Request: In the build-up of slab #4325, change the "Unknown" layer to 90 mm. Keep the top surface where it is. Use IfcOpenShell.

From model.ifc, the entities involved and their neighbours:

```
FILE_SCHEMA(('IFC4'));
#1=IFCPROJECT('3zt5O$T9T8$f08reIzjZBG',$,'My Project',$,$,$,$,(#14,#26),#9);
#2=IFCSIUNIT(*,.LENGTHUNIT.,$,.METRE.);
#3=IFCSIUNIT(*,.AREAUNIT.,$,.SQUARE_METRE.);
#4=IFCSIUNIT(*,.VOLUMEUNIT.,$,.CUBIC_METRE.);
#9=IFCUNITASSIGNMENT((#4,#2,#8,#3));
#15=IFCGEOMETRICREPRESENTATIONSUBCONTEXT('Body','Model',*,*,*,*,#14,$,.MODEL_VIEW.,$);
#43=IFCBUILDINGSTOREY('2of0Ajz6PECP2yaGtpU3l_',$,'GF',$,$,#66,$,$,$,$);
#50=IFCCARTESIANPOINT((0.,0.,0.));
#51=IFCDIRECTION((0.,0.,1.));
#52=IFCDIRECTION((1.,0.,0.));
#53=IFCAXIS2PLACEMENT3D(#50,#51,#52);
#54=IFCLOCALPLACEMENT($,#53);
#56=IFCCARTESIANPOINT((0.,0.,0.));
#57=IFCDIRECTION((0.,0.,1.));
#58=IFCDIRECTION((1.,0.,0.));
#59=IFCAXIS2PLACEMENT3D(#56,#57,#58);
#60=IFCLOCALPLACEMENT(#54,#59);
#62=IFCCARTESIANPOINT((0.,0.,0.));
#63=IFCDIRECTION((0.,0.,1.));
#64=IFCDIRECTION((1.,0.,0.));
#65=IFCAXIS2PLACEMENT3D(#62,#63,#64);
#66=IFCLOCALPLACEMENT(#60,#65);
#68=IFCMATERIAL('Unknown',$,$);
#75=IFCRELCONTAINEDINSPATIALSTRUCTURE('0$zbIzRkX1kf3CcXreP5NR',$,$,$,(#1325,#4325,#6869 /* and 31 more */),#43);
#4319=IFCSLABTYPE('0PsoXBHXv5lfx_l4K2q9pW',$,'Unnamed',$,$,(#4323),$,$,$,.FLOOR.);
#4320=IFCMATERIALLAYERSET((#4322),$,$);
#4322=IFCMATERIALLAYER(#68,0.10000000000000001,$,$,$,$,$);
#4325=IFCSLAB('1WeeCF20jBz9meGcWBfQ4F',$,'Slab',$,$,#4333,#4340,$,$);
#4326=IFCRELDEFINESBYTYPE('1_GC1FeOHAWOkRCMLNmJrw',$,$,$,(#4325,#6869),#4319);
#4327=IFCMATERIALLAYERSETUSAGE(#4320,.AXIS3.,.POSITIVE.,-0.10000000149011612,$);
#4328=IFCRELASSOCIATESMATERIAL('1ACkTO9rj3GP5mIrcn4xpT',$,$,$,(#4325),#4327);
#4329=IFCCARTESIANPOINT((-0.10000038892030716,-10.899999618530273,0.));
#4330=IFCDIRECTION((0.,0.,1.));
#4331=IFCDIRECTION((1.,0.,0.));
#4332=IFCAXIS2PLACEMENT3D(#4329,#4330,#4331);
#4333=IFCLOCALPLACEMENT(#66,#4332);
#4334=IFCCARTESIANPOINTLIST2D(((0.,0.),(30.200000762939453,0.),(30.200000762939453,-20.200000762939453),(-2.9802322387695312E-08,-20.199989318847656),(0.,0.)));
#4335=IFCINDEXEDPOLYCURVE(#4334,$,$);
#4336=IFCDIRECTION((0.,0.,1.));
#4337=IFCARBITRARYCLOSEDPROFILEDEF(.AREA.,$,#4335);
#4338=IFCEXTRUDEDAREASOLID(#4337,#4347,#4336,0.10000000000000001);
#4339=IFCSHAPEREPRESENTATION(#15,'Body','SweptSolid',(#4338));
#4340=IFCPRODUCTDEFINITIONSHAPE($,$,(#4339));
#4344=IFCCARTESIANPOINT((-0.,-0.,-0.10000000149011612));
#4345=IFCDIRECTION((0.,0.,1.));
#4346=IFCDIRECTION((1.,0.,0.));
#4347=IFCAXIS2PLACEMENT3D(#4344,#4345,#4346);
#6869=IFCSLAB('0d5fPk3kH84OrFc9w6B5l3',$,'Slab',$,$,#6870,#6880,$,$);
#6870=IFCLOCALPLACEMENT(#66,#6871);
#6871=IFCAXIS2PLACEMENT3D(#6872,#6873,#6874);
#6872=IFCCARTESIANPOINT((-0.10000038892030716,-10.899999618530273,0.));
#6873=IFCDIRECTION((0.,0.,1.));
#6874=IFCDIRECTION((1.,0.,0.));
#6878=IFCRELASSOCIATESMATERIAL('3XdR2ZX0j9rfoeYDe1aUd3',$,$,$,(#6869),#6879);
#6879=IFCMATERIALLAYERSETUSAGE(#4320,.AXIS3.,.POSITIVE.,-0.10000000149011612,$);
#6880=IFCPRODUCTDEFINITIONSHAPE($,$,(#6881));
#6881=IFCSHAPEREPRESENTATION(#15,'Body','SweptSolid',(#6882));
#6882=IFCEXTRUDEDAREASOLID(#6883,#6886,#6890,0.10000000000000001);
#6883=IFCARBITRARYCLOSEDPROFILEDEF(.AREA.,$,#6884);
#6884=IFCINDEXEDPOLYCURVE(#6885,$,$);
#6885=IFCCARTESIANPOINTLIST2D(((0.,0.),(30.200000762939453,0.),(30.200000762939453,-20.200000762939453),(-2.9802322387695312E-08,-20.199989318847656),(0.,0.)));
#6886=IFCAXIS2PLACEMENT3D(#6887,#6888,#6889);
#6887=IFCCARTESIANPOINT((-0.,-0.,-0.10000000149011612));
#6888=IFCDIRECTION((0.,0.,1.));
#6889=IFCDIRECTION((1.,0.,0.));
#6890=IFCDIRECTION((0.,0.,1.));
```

```python
import ifcopenshell
import ifcopenshell.util.element
import ifcopenshell.util.representation
import ifcopenshell.util.unit

model = ifcopenshell.open("model.ifc")
unit_scale = ifcopenshell.util.unit.calculate_unit_scale(model)

layer_set = model.by_id(4320)
layer = next(l for l in layer_set.MaterialLayers if l.Material and l.Material.Name == "Unknown")
change = 0.09 / unit_scale - layer.LayerThickness
layer.LayerThickness += change

# The layer set is shared, so every slab that uses it gets the new thickness.
slabs = [e for e in ifcopenshell.util.element.get_elements_by_material(model, layer_set) if e.is_a("IfcSlab")]
for slab in sorted(slabs, key=lambda e: e.id()):
    body = ifcopenshell.util.representation.get_representation(slab, "Model", "Body")
    solid = body.Items[0]
    old_depth = solid.Depth
    solid.Depth += change
    # Extruded upwards: lower the start of the extrusion so the top stays.
    x, y, z = solid.Position.Location.Coordinates
    solid.Position.Location = model.createIfcCartesianPoint((x, y, z - change))
    print(slab.id(), f"{old_depth:g} -> {solid.Depth:g}")

# The layers are counted up from the underside, which has moved.
for usage in {ifcopenshell.util.element.get_material(slab) for slab in slabs}:
    usage.OffsetFromReferenceLine -= change

model.write("model_edited.ifc")
```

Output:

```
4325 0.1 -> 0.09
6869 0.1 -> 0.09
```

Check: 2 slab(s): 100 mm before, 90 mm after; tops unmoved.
